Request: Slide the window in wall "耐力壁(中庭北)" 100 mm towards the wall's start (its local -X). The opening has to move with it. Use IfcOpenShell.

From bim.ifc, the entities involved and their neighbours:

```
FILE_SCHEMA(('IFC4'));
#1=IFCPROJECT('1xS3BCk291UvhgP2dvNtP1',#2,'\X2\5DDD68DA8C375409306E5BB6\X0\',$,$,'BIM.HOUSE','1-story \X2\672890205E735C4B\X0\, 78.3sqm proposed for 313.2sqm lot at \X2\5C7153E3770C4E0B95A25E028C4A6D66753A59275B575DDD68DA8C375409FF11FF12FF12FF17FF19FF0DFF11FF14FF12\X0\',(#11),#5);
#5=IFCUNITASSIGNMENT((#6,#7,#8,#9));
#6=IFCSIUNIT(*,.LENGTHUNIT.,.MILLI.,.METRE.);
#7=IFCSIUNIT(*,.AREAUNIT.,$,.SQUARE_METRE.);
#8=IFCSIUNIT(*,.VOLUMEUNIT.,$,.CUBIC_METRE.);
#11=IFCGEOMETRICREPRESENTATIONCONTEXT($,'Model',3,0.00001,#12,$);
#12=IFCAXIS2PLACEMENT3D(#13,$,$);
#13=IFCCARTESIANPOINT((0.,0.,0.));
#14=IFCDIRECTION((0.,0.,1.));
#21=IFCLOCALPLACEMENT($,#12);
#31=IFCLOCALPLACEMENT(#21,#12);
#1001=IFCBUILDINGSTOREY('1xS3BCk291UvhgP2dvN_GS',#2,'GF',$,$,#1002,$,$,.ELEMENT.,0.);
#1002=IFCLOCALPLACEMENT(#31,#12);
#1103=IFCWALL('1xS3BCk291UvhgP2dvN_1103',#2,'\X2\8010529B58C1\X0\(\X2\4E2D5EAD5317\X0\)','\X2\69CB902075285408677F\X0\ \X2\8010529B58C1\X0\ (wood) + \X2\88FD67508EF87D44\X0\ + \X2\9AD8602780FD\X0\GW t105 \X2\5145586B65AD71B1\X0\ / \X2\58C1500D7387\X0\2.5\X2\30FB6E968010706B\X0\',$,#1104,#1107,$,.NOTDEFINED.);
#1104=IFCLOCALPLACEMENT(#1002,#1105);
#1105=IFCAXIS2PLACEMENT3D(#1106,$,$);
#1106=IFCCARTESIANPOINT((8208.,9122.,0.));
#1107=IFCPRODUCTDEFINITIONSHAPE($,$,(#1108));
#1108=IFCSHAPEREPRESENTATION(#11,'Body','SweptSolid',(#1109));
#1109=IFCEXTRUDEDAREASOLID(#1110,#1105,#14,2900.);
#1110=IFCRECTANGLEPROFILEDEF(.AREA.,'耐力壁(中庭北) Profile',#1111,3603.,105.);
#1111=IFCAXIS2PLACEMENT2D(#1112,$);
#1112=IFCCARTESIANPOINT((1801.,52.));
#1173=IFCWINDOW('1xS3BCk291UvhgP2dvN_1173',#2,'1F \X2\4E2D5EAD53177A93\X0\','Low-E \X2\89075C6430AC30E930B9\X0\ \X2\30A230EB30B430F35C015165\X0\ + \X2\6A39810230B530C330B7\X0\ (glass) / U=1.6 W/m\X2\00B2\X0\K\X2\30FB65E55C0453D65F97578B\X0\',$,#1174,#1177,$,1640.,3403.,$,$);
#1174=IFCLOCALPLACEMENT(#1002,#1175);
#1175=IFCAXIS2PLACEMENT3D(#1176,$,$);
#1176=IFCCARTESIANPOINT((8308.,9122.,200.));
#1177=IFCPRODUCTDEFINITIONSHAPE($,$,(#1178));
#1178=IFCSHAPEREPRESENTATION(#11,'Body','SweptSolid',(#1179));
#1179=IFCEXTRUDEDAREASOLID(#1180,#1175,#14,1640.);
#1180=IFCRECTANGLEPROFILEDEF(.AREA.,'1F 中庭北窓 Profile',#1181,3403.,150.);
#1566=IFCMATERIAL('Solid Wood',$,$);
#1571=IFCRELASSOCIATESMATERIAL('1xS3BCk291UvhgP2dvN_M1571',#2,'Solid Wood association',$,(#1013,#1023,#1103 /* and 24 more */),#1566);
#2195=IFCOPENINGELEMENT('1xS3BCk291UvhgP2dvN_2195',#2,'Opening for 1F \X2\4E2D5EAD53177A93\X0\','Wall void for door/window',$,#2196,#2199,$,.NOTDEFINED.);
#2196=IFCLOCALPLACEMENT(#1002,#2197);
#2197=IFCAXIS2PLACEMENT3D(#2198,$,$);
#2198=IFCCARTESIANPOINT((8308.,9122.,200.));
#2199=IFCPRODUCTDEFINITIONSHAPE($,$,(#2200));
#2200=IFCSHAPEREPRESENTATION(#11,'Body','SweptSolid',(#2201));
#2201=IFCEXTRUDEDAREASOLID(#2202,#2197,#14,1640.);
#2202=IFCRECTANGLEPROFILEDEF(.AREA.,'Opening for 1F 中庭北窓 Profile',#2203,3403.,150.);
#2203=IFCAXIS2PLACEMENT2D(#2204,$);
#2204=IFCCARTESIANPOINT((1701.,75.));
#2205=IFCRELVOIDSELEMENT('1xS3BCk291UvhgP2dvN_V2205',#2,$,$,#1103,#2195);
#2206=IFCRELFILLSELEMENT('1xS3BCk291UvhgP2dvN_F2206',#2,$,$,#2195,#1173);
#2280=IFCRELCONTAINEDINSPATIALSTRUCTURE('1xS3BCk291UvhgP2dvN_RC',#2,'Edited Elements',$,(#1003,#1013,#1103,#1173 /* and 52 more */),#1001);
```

```python
import ifcopenshell
import ifcopenshell.api.geometry
import ifcopenshell.util.placement

model = ifcopenshell.open("bim.ifc")

window = model.by_id(1173)
opening = window.FillsVoids[0].RelatingOpeningElement
wall = opening.VoidsElements[0].RelatingBuildingElement

wall_matrix = ifcopenshell.util.placement.get_local_placement(wall.ObjectPlacement)
shift = wall_matrix[:3, 0] * -100.0
before = ifcopenshell.util.placement.get_local_placement(window.ObjectPlacement)[:3, 3].copy()

# The window is not placed relative to its opening, so move both.
for product in (opening, window):
    matrix = ifcopenshell.util.placement.get_local_placement(product.ObjectPlacement)
    matrix[:3, 3] += shift
    ifcopenshell.api.geometry.edit_object_placement(model, product=product, matrix=matrix, is_si=False)

after = ifcopenshell.util.placement.get_local_placement(window.ObjectPlacement)[:3, 3]
print("window moved by", (after - before).round(3) + 0.0)

model.write("bim_edited.ifc")
```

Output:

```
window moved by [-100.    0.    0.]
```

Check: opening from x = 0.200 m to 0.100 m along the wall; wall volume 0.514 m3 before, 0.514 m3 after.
